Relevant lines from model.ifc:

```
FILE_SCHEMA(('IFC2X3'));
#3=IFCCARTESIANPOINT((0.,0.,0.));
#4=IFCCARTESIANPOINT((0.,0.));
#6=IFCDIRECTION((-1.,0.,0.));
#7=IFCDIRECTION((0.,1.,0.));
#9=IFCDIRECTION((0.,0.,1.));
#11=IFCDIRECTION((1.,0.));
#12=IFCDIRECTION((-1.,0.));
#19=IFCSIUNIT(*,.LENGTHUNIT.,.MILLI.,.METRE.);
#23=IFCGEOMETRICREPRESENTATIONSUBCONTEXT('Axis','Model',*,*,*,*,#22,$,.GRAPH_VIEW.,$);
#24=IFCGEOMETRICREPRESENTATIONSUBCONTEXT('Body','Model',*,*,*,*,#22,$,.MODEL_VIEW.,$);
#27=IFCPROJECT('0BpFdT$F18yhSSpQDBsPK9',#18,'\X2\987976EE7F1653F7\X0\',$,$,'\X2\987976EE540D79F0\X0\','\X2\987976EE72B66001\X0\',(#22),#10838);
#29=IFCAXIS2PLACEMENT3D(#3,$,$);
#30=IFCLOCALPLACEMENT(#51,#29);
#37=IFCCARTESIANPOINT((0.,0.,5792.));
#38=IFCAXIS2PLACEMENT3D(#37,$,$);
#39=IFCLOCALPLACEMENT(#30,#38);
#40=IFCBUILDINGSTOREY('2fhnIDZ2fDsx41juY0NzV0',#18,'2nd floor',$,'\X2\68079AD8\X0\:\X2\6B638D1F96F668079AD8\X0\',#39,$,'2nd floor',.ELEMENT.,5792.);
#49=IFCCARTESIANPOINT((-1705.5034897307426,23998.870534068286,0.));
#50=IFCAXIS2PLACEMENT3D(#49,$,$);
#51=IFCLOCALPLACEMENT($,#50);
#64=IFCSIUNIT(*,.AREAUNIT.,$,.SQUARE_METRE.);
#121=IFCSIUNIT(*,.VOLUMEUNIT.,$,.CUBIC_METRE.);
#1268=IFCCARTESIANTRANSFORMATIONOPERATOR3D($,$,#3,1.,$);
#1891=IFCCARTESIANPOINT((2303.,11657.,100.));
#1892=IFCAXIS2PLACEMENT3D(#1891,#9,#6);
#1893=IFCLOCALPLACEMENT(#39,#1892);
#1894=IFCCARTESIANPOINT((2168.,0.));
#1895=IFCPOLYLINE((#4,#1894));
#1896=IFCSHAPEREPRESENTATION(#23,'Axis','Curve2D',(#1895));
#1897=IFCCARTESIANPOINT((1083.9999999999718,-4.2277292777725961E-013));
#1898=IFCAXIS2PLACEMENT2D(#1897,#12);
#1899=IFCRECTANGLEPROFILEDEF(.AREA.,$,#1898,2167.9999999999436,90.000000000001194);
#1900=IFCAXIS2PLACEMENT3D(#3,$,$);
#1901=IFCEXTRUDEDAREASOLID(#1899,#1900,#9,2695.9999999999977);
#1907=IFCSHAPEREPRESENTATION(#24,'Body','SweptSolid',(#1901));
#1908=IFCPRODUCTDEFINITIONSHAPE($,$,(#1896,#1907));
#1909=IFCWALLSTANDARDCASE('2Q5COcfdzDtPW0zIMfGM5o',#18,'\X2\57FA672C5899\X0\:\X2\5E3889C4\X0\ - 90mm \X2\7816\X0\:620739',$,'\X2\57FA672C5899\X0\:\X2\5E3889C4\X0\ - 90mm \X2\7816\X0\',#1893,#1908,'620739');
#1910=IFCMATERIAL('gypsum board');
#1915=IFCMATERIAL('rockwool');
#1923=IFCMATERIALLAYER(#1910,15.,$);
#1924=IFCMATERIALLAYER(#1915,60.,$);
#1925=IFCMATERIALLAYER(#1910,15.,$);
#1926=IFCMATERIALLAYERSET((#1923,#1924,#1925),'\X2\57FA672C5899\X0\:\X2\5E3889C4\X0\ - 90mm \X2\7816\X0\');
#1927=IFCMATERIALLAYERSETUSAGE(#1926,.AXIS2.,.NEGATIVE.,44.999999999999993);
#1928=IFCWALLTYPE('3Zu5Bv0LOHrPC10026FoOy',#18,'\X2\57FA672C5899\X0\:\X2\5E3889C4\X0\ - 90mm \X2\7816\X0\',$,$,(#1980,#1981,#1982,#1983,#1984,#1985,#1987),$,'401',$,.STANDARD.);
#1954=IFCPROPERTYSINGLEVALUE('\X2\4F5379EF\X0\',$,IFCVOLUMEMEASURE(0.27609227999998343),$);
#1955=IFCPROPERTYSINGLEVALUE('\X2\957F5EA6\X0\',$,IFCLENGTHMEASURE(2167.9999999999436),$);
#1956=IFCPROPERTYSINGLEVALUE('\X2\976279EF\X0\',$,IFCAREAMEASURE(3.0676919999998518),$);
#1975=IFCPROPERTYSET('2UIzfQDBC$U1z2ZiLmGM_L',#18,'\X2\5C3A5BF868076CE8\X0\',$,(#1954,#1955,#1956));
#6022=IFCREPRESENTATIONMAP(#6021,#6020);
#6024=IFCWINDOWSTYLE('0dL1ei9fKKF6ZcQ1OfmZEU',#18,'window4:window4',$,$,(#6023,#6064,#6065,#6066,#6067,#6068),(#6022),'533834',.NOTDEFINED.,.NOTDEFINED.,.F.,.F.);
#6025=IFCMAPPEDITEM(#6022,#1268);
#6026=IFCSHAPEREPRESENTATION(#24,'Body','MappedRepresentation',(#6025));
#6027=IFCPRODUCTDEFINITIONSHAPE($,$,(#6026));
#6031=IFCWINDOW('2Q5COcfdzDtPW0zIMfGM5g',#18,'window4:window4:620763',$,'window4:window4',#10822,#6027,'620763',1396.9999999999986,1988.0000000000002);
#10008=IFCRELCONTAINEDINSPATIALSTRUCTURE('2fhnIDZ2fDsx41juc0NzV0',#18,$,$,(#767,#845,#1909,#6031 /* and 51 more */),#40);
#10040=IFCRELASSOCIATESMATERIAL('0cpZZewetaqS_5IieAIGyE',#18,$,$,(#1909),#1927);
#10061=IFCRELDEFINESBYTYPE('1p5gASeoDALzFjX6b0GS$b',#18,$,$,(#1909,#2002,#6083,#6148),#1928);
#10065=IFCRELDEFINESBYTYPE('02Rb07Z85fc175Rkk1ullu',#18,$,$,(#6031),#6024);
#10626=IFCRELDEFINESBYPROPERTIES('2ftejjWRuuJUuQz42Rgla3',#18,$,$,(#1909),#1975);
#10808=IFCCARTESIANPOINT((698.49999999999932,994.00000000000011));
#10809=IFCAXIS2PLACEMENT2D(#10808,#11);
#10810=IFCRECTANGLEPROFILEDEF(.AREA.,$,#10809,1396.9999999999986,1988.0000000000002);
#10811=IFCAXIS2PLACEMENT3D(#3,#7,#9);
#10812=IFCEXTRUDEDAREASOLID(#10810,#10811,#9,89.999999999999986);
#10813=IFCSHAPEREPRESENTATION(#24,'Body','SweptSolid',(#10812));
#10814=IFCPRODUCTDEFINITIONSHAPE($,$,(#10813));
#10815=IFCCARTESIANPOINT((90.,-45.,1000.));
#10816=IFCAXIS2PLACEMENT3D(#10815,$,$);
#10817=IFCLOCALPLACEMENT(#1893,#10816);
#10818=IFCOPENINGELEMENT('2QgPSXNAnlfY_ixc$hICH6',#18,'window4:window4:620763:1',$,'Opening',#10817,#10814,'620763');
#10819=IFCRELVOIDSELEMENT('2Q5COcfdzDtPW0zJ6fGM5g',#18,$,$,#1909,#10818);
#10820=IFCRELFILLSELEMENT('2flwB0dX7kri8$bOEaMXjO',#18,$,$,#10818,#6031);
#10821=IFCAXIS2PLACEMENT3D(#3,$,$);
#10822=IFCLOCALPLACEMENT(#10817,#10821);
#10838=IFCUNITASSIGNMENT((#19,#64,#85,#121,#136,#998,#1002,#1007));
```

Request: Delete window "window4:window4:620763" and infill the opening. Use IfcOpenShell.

```python
import ifcopenshell
import ifcopenshell.api.feature
import ifcopenshell.api.pset
import ifcopenshell.api.root
import ifcopenshell.geom
import ifcopenshell.util.element
import ifcopenshell.util.shape
import ifcopenshell.util.unit

model = ifcopenshell.open("model.ifc")
area_scale = ifcopenshell.util.unit.calculate_unit_scale(model, "AREAUNIT")
volume_scale = ifcopenshell.util.unit.calculate_unit_scale(model, "VOLUMEUNIT")
settings = ifcopenshell.geom.settings()


def volume(element):
    """Net volume in cubic metres, openings subtracted."""
    shape = ifcopenshell.geom.create_shape(settings, element)
    return ifcopenshell.util.shape.get_volume(shape.geometry)


window = model.by_guid("2Q5COcfdzDtPW0zIMfGM5g")
opening = window.FillsVoids[0].RelatingOpeningElement
wall = opening.VoidsElements[0].RelatingBuildingElement
before = volume(wall)

ifcopenshell.api.root.remove_product(model, product=window)
ifcopenshell.api.feature.remove_feature(model, feature=opening)

after = volume(wall)
thickness = 0.09  # wall thickness in metres

# Update the wall's stored quantities.
pset = model.by_id(ifcopenshell.util.element.get_pset(wall, "尺寸标注", should_inherit=False)["id"])
ifcopenshell.api.pset.edit_pset(model, pset=pset, properties={
    "体积": model.create_entity("IfcVolumeMeasure", after / volume_scale),
    "面积": model.create_entity("IfcAreaMeasure", after / thickness / area_scale),
})

print(f"wall volume {before:.3f} -> {after:.3f} m3")

model.write("model_updated.ifc")
```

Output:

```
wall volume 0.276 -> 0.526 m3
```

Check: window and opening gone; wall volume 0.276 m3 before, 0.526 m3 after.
